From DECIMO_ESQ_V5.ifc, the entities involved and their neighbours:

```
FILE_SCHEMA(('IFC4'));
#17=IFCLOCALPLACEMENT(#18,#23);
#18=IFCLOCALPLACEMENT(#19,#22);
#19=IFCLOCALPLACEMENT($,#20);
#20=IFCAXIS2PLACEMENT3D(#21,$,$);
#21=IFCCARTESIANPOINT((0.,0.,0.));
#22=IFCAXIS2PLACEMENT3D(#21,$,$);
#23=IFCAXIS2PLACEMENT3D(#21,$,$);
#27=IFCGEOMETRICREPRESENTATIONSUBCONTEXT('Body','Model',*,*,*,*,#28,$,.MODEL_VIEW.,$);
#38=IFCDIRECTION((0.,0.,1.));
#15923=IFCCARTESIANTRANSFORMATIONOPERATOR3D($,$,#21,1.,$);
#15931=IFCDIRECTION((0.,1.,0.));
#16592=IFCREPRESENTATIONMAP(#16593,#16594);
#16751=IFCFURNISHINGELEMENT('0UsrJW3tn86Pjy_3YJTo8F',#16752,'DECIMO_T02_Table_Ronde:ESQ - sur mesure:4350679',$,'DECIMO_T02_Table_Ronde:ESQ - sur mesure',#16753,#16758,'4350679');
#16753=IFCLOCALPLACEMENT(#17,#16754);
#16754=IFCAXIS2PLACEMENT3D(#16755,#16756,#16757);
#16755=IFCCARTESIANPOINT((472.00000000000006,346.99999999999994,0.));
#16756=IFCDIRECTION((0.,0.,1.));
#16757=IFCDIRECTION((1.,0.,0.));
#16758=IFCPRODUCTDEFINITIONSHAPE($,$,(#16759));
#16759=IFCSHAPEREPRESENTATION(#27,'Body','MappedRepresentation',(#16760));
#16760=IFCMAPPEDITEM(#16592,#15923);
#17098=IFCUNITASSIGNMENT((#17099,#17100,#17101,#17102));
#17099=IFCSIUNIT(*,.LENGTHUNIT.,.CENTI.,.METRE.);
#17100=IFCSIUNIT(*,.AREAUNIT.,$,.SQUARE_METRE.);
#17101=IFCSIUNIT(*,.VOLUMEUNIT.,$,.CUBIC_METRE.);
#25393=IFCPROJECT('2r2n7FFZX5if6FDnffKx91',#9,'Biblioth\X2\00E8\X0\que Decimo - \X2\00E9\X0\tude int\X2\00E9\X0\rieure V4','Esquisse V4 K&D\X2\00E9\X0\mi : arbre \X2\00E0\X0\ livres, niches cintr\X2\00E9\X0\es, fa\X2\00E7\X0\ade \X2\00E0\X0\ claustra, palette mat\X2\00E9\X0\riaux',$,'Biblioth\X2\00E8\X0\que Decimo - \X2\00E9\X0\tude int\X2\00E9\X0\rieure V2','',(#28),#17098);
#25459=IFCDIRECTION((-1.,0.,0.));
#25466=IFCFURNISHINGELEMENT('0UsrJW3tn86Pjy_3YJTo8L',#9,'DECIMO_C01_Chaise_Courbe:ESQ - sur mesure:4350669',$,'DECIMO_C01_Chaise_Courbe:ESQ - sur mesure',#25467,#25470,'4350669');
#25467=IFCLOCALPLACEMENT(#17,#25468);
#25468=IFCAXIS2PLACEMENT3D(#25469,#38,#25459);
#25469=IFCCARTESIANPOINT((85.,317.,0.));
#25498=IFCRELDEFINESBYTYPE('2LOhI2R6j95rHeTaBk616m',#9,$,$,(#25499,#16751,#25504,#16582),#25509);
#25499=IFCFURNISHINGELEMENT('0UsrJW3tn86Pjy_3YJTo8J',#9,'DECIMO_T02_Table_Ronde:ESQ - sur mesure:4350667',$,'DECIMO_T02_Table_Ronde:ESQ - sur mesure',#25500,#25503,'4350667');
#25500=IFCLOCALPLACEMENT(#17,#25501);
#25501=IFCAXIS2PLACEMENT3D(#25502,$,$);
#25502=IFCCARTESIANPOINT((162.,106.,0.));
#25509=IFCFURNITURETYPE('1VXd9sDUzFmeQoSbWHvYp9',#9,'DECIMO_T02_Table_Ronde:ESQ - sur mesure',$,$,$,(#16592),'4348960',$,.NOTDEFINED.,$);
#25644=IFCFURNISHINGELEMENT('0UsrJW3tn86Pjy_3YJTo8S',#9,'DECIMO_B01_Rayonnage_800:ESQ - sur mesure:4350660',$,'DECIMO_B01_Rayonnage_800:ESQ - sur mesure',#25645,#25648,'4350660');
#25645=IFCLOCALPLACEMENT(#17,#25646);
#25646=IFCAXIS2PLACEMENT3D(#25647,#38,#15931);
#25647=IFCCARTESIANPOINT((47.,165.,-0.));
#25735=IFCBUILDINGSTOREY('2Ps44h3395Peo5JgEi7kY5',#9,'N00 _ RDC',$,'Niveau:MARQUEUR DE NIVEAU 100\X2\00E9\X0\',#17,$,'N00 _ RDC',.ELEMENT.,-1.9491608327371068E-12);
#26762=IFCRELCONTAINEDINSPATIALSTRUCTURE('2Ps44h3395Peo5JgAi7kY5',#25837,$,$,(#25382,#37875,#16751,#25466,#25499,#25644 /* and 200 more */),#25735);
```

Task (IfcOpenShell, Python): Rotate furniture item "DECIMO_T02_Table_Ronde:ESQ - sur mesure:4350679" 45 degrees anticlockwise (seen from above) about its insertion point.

```python
import ifcopenshell
import ifcopenshell.api.geometry
import ifcopenshell.util.placement

model = ifcopenshell.open("DECIMO_ESQ_V5.ifc")

item = model.by_guid("0UsrJW3tn86Pjy_3YJTo8F")
matrix = ifcopenshell.util.placement.get_local_placement(item.ObjectPlacement)
matrix = matrix @ ifcopenshell.util.placement.rotation(45, "Z")
ifcopenshell.api.geometry.edit_object_placement(model, product=item, matrix=matrix, is_si=False)

print(ifcopenshell.util.placement.get_local_placement(item.ObjectPlacement).round(3) + 0.0)

model.write("DECIMO_ESQ_V5_edited.ifc")
```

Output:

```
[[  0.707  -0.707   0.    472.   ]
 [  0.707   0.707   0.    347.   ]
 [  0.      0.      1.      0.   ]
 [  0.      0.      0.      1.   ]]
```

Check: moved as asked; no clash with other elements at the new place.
